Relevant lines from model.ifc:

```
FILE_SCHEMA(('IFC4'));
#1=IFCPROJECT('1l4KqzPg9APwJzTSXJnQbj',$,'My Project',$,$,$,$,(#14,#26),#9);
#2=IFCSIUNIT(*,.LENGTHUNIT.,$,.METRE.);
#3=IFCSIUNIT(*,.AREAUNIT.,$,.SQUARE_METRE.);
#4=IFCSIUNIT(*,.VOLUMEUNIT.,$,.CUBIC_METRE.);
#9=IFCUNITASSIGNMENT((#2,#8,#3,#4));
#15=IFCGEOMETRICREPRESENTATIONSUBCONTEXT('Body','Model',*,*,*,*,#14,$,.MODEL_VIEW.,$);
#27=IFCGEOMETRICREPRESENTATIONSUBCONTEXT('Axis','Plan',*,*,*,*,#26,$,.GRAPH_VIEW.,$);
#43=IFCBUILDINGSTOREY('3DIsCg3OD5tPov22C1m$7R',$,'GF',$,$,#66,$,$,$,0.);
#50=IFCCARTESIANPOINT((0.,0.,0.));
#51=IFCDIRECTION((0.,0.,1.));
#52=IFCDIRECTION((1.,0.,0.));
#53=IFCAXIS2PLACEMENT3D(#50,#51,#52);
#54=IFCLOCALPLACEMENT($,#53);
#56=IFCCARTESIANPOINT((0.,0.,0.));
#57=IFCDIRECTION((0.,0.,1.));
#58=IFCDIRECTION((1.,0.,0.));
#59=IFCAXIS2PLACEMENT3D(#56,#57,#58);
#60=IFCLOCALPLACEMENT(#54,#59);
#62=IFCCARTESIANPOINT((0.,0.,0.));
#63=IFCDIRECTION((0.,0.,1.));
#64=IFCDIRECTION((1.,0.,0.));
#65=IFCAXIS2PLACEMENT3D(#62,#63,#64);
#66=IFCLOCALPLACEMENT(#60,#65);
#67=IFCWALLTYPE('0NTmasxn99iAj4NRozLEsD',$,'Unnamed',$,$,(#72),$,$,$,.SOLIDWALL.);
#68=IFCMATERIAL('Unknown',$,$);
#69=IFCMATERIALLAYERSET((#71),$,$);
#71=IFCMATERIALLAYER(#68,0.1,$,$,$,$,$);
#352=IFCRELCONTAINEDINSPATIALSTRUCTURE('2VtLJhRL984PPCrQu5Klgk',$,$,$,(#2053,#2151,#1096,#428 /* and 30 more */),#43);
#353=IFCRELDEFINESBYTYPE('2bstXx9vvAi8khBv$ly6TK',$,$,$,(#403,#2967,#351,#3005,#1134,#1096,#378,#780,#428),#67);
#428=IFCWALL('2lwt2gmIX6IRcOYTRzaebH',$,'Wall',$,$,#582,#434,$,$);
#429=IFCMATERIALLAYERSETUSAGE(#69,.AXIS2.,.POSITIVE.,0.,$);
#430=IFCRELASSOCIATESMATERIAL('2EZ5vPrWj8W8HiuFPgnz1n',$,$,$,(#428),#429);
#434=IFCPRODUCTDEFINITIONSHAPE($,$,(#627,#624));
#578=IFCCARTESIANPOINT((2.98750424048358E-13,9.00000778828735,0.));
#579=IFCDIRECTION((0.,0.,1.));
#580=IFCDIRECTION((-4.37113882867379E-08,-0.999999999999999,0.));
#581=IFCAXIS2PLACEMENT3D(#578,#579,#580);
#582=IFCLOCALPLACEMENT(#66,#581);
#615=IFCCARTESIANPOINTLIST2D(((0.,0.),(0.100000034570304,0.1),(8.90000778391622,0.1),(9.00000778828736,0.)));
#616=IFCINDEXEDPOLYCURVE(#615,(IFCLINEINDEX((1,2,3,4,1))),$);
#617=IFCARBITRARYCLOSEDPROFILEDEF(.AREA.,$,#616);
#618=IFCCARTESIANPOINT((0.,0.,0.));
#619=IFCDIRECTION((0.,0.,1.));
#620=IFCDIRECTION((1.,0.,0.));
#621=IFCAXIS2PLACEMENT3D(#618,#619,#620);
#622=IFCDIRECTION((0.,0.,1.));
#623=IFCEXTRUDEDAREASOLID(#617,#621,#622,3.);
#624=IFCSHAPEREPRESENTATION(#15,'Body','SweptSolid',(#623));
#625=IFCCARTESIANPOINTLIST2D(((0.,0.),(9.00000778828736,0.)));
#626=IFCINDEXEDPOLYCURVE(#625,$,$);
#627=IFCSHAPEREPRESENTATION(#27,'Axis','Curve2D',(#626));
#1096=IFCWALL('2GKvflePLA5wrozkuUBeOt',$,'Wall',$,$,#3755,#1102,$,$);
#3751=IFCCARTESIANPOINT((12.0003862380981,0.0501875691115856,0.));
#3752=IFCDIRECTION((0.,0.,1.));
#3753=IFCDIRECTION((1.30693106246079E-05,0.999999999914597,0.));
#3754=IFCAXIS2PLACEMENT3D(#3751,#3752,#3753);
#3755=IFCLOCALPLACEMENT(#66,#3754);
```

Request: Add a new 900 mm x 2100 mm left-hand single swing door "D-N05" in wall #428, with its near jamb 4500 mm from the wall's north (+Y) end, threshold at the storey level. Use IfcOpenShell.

```python
import numpy as np
import ifcopenshell
import ifcopenshell.api.feature
import ifcopenshell.api.geometry
import ifcopenshell.api.root
import ifcopenshell.api.spatial
import ifcopenshell.geom
import ifcopenshell.util.element
import ifcopenshell.util.placement
import ifcopenshell.util.representation
import ifcopenshell.util.shape
import ifcopenshell.util.unit

model = ifcopenshell.open("model.ifc")
unit_scale = ifcopenshell.util.unit.calculate_unit_scale(model)
settings = ifcopenshell.geom.settings()


def volume(element):
    """Net volume in cubic metres, openings subtracted."""
    shape = ifcopenshell.geom.create_shape(settings, element)
    return ifcopenshell.util.shape.get_volume(shape.geometry)


wall = model.by_guid("2lwt2gmIX6IRcOYTRzaebH")
storey = ifcopenshell.util.element.get_container(wall, ifc_class="IfcBuildingStorey")
context = ifcopenshell.util.representation.get_context(model, "Model", "Body", "MODEL_VIEW")
before = volume(wall)

width, height, from_end, sill = 0.9, 2.1, 4.5, 0.0  # metres

# The wall runs along its own X axis, and the end named is its -X end.
wall_shape = ifcopenshell.geom.create_shape(settings, wall)
x, y, z = ifcopenshell.util.shape.get_vertices(wall_shape.geometry).T
start = x.min() + from_end
face, thickness = float(y.min()), float(y.max() - y.min())
wall_matrix = ifcopenshell.util.placement.get_local_placement(wall.ObjectPlacement)
level = ifcopenshell.util.placement.get_local_placement(storey.ObjectPlacement)[2, 3]


def in_wall(x, y):
    """Placement at x, y metres in the wall's axes, at sill height."""
    matrix = wall_matrix.copy()
    matrix[:, 3] = wall_matrix @ np.array([x / unit_scale, y / unit_scale, 0.0, 1.0])
    matrix[2, 3] = level + sill / unit_scale
    return matrix


# Opening: a box that overshoots both wall faces by 50 mm.
opening = ifcopenshell.api.root.create_entity(model, ifc_class="IfcOpeningElement", predefined_type="OPENING")
box = ifcopenshell.api.geometry.add_wall_representation(
    model, context=context, length=width, height=height, thickness=thickness + 0.1
)
ifcopenshell.api.geometry.assign_representation(model, product=opening, representation=box)
ifcopenshell.api.geometry.edit_object_placement(model, product=opening, matrix=in_wall(start, face - 0.05), is_si=False)
ifcopenshell.api.feature.add_feature(model, feature=opening, element=wall)

door = ifcopenshell.api.root.create_entity(model, ifc_class="IfcDoor", name="D-N05", predefined_type="DOOR")
door.OverallWidth, door.OverallHeight = width / unit_scale, height / unit_scale
door.OperationType = "SINGLE_SWING_LEFT"
body = ifcopenshell.api.geometry.add_door_representation(
    model,
    context=context,
    overall_width=door.OverallWidth,
    overall_height=door.OverallHeight,
    operation_type="SINGLE_SWING_LEFT",
    lining_properties={"LiningDepth": thickness / unit_scale, "ThresholdDepth": thickness / unit_scale},
)
ifcopenshell.api.geometry.assign_representation(model, product=door, representation=body)
ifcopenshell.api.spatial.assign_container(model, products=[door], relating_structure=storey)
ifcopenshell.api.feature.add_filling(model, opening=opening, element=door)

# The lining spans the wall, so the door starts at the wall face.
ifcopenshell.api.geometry.edit_object_placement(model, product=door, matrix=in_wall(start, face), is_si=False)

after = volume(wall)

print(f"wall volume {before:.3f} -> {after:.3f} m3")

model.write("model_updated.ifc")
```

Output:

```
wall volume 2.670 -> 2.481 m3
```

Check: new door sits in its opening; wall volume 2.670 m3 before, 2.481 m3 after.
